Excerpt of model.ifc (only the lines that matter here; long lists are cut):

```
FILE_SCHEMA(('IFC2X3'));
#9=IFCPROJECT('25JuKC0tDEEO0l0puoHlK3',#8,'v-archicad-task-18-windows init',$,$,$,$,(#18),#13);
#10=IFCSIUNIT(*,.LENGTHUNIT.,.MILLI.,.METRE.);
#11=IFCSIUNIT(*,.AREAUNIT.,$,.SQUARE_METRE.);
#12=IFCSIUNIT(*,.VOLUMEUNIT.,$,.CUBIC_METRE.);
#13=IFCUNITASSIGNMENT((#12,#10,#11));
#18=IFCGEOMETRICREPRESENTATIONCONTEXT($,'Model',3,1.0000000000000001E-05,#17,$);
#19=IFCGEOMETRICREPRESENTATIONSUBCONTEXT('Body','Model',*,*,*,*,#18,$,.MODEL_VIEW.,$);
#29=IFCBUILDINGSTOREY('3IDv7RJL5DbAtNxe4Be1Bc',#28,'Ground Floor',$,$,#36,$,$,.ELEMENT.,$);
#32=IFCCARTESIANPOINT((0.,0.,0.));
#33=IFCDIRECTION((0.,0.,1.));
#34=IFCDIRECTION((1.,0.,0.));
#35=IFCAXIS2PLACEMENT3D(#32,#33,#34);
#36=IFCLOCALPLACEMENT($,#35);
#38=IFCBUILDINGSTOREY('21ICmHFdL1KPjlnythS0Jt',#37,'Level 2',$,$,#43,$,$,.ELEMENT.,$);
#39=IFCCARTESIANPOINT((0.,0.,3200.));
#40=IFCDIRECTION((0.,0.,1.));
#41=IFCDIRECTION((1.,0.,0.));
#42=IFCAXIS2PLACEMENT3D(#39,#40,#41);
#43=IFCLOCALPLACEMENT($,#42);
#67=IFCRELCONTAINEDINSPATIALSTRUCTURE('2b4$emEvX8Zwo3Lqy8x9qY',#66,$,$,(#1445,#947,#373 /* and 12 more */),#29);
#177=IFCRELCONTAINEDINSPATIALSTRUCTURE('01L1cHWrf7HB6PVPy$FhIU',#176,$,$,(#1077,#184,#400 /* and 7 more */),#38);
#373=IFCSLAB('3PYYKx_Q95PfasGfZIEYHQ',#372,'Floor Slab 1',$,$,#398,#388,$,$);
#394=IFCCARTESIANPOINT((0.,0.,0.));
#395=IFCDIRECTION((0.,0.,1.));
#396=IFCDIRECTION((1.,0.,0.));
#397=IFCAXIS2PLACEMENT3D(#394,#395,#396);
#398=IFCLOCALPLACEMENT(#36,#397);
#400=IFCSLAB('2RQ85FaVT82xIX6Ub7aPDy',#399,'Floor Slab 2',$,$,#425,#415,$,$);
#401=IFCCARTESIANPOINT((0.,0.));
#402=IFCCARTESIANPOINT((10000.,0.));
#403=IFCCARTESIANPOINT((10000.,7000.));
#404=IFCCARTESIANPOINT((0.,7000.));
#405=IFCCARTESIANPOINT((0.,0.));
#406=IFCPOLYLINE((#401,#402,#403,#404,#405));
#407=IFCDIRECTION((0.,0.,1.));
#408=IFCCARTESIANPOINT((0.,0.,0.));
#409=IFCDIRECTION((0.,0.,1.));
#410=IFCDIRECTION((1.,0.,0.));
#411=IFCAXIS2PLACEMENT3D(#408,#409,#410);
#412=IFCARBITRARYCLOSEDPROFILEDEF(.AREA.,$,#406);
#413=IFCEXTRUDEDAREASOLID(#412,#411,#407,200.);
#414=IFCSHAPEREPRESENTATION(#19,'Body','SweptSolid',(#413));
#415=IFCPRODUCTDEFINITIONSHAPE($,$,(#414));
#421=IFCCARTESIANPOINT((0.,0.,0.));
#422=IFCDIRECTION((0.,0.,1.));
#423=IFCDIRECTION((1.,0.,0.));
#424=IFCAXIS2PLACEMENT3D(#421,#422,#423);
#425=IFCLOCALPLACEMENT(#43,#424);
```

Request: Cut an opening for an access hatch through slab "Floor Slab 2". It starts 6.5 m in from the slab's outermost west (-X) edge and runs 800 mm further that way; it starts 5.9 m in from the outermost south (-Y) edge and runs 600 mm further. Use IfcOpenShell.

```python
import numpy as np
import ifcopenshell
import ifcopenshell.api.feature
import ifcopenshell.api.geometry
import ifcopenshell.api.root
import ifcopenshell.geom
import ifcopenshell.util.placement
import ifcopenshell.util.representation
import ifcopenshell.util.shape
import ifcopenshell.util.unit

model = ifcopenshell.open("model.ifc")
unit_scale = ifcopenshell.util.unit.calculate_unit_scale(model)
settings = ifcopenshell.geom.settings()


def volume(element):
    """Net volume in cubic metres, openings subtracted."""
    shape = ifcopenshell.geom.create_shape(settings, element)
    return ifcopenshell.util.shape.get_volume(shape.geometry)


slab = model.by_guid("2RQ85FaVT82xIX6Ub7aPDy")
before = volume(slab)

# Extent in the slab's own axes, in metres. The edges named are its -X and -Y sides.
slab_shape = ifcopenshell.geom.create_shape(settings, slab)
vertices = ifcopenshell.util.shape.get_vertices(slab_shape.geometry)
x_min, y_min, bottom = vertices.min(axis=0)
top = vertices[:, 2].max()

opening = ifcopenshell.api.root.create_entity(model, ifc_class="IfcOpeningElement", name="Access hatch opening")
context = ifcopenshell.util.representation.get_context(model, "Model", "Body", "MODEL_VIEW")
width, depth = 0.8, 0.6
outline = [(0.0, 0.0), (width, 0.0), (width, depth), (0.0, depth), (0.0, 0.0)]
# Overshoot both faces by 50 mm so the cut is clean.
shape = ifcopenshell.api.geometry.add_slab_representation(
    model, context=context, depth=top - bottom + 0.1, polyline=outline
)
ifcopenshell.api.geometry.assign_representation(model, product=opening, representation=shape)

matrix = ifcopenshell.util.placement.get_local_placement(slab.ObjectPlacement)
matrix[:, 3] = matrix @ np.append(np.array([x_min + 6.5, y_min + 5.9, bottom - 0.05]) / unit_scale, 1.0)
ifcopenshell.api.geometry.edit_object_placement(model, product=opening, matrix=matrix, is_si=False)
ifcopenshell.api.feature.add_feature(model, feature=opening, element=slab)

after = volume(slab)

print(f"slab volume {before:.3f} -> {after:.3f} m3")

model.write("model_updated.ifc")
```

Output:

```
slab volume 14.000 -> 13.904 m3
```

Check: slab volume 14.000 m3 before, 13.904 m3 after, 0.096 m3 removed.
